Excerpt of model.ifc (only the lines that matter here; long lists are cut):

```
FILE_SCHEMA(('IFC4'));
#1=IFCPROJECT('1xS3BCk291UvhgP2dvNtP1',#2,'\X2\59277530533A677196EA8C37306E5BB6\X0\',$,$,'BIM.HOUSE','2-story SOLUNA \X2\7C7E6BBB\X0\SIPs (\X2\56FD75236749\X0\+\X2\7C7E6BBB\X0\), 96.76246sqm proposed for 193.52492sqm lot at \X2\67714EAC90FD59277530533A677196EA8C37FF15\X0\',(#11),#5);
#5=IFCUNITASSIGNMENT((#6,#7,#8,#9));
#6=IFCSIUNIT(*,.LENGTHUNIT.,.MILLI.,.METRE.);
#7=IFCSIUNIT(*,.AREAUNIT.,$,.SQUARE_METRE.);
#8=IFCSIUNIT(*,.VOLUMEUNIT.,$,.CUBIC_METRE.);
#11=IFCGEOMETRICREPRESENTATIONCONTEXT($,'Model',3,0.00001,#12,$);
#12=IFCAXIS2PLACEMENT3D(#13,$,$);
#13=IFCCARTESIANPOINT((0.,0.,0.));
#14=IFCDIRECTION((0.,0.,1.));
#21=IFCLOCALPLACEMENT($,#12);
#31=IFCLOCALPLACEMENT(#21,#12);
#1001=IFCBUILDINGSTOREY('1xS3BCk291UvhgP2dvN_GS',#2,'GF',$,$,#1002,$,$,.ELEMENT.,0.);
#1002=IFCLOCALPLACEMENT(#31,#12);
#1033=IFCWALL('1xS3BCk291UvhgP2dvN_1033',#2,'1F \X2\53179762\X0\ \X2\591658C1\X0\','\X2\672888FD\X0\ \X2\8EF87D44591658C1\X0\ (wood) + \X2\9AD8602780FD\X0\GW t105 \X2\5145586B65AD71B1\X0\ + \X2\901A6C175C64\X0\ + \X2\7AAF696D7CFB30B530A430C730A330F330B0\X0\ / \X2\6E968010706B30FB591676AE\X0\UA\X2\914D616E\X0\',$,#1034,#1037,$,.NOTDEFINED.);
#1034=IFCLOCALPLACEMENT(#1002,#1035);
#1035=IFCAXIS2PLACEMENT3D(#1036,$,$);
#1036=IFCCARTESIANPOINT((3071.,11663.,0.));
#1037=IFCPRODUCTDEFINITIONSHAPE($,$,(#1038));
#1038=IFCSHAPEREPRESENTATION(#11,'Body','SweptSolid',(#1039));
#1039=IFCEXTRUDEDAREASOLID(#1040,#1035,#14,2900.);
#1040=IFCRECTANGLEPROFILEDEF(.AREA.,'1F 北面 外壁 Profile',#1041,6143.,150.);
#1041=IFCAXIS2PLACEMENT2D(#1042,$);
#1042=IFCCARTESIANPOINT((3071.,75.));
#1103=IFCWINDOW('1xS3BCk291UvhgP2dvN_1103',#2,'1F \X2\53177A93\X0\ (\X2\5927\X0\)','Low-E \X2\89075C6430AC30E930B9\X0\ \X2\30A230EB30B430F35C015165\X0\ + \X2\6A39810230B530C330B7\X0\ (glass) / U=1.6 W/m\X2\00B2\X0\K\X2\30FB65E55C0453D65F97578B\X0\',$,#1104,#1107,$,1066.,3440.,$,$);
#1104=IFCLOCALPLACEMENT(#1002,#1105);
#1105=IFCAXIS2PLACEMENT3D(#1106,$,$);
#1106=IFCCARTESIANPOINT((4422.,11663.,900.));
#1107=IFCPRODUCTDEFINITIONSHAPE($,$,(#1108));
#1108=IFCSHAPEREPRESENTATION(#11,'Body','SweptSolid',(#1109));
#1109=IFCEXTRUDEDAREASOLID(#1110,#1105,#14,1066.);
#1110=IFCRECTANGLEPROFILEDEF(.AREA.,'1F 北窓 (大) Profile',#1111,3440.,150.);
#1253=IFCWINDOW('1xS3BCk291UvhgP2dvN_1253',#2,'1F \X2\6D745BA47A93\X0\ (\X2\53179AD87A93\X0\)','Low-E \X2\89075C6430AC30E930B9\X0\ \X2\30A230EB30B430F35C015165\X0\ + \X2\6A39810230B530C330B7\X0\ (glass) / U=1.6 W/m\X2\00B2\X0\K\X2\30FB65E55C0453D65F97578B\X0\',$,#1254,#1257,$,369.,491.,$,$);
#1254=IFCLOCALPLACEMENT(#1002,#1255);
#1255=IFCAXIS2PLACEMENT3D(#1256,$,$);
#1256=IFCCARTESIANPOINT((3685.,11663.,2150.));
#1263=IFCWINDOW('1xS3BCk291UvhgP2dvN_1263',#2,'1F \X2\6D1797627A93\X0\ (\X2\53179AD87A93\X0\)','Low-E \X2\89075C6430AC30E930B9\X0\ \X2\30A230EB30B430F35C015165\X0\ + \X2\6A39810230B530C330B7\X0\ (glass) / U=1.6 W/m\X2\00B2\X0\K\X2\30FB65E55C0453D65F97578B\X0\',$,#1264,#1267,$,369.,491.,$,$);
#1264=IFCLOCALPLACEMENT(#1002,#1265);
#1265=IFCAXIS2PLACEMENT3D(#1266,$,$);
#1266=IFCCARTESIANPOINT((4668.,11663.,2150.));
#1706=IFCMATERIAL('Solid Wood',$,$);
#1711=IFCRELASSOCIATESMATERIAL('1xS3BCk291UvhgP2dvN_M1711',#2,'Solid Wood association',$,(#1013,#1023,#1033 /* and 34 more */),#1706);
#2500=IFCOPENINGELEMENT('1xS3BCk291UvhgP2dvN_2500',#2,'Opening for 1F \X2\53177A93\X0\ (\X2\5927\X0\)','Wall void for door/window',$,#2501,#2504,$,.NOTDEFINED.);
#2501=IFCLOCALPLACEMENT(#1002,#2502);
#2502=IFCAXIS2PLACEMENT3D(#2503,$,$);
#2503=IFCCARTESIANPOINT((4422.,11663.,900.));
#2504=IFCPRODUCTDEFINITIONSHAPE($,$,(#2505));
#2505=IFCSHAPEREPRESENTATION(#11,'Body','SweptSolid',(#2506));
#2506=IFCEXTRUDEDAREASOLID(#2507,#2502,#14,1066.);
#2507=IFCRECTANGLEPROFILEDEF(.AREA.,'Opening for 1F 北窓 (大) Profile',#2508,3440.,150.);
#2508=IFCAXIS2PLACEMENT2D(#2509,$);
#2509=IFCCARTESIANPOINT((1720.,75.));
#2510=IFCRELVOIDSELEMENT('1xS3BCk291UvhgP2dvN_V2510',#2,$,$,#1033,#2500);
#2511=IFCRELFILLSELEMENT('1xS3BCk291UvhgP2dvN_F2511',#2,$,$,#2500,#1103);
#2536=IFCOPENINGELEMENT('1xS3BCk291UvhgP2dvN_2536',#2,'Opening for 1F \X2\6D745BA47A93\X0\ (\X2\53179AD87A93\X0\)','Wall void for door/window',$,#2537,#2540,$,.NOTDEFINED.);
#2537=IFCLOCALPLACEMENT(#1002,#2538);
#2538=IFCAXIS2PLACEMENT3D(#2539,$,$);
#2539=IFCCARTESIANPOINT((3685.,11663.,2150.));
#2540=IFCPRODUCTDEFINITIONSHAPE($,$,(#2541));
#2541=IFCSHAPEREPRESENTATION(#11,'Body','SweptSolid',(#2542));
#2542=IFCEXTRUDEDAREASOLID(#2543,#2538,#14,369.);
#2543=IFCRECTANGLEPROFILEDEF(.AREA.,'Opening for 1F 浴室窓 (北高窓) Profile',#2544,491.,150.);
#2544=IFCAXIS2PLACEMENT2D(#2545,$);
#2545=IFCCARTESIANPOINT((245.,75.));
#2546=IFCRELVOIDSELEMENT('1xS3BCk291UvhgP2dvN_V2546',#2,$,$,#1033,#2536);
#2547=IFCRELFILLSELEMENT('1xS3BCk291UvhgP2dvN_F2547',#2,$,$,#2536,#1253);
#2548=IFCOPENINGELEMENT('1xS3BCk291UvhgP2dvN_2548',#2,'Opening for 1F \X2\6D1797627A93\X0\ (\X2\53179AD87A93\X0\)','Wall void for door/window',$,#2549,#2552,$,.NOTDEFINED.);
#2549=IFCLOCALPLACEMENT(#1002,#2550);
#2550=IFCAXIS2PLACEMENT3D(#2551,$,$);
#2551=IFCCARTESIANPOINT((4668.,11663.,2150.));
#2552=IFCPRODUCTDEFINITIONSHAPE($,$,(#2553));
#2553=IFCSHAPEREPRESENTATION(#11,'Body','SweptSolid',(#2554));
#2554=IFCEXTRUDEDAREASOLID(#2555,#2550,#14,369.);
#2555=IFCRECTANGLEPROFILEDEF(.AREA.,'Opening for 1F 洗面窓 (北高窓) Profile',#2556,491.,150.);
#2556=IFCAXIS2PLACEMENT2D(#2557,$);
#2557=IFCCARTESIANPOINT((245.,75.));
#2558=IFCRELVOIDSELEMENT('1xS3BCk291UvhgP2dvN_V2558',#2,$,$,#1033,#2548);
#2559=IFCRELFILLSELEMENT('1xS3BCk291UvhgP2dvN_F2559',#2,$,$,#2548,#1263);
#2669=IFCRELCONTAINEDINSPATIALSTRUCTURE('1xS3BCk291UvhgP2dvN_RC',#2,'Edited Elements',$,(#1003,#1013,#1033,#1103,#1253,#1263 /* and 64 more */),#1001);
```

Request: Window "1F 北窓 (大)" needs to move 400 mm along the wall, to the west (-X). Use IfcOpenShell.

```python
import ifcopenshell
import ifcopenshell.api.geometry
import ifcopenshell.util.placement

model = ifcopenshell.open("model.ifc")

window = model.by_guid("1xS3BCk291UvhgP2dvN_1103")
opening = window.FillsVoids[0].RelatingOpeningElement
wall = opening.VoidsElements[0].RelatingBuildingElement

wall_matrix = ifcopenshell.util.placement.get_local_placement(wall.ObjectPlacement)
shift = wall_matrix[:3, 0] * -400.0
before = ifcopenshell.util.placement.get_local_placement(window.ObjectPlacement)[:3, 3].copy()

# The window is not placed relative to its opening, so move both.
for product in (opening, window):
    matrix = ifcopenshell.util.placement.get_local_placement(product.ObjectPlacement)
    matrix[:3, 3] += shift
    ifcopenshell.api.geometry.edit_object_placement(model, product=product, matrix=matrix, is_si=False)

after = ifcopenshell.util.placement.get_local_placement(window.ObjectPlacement)[:3, 3]
print("window moved by", (after - before).round(3) + 0.0)

model.write("model_edited.ifc")
```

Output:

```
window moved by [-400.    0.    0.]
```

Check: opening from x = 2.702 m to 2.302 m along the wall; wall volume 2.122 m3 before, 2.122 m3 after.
